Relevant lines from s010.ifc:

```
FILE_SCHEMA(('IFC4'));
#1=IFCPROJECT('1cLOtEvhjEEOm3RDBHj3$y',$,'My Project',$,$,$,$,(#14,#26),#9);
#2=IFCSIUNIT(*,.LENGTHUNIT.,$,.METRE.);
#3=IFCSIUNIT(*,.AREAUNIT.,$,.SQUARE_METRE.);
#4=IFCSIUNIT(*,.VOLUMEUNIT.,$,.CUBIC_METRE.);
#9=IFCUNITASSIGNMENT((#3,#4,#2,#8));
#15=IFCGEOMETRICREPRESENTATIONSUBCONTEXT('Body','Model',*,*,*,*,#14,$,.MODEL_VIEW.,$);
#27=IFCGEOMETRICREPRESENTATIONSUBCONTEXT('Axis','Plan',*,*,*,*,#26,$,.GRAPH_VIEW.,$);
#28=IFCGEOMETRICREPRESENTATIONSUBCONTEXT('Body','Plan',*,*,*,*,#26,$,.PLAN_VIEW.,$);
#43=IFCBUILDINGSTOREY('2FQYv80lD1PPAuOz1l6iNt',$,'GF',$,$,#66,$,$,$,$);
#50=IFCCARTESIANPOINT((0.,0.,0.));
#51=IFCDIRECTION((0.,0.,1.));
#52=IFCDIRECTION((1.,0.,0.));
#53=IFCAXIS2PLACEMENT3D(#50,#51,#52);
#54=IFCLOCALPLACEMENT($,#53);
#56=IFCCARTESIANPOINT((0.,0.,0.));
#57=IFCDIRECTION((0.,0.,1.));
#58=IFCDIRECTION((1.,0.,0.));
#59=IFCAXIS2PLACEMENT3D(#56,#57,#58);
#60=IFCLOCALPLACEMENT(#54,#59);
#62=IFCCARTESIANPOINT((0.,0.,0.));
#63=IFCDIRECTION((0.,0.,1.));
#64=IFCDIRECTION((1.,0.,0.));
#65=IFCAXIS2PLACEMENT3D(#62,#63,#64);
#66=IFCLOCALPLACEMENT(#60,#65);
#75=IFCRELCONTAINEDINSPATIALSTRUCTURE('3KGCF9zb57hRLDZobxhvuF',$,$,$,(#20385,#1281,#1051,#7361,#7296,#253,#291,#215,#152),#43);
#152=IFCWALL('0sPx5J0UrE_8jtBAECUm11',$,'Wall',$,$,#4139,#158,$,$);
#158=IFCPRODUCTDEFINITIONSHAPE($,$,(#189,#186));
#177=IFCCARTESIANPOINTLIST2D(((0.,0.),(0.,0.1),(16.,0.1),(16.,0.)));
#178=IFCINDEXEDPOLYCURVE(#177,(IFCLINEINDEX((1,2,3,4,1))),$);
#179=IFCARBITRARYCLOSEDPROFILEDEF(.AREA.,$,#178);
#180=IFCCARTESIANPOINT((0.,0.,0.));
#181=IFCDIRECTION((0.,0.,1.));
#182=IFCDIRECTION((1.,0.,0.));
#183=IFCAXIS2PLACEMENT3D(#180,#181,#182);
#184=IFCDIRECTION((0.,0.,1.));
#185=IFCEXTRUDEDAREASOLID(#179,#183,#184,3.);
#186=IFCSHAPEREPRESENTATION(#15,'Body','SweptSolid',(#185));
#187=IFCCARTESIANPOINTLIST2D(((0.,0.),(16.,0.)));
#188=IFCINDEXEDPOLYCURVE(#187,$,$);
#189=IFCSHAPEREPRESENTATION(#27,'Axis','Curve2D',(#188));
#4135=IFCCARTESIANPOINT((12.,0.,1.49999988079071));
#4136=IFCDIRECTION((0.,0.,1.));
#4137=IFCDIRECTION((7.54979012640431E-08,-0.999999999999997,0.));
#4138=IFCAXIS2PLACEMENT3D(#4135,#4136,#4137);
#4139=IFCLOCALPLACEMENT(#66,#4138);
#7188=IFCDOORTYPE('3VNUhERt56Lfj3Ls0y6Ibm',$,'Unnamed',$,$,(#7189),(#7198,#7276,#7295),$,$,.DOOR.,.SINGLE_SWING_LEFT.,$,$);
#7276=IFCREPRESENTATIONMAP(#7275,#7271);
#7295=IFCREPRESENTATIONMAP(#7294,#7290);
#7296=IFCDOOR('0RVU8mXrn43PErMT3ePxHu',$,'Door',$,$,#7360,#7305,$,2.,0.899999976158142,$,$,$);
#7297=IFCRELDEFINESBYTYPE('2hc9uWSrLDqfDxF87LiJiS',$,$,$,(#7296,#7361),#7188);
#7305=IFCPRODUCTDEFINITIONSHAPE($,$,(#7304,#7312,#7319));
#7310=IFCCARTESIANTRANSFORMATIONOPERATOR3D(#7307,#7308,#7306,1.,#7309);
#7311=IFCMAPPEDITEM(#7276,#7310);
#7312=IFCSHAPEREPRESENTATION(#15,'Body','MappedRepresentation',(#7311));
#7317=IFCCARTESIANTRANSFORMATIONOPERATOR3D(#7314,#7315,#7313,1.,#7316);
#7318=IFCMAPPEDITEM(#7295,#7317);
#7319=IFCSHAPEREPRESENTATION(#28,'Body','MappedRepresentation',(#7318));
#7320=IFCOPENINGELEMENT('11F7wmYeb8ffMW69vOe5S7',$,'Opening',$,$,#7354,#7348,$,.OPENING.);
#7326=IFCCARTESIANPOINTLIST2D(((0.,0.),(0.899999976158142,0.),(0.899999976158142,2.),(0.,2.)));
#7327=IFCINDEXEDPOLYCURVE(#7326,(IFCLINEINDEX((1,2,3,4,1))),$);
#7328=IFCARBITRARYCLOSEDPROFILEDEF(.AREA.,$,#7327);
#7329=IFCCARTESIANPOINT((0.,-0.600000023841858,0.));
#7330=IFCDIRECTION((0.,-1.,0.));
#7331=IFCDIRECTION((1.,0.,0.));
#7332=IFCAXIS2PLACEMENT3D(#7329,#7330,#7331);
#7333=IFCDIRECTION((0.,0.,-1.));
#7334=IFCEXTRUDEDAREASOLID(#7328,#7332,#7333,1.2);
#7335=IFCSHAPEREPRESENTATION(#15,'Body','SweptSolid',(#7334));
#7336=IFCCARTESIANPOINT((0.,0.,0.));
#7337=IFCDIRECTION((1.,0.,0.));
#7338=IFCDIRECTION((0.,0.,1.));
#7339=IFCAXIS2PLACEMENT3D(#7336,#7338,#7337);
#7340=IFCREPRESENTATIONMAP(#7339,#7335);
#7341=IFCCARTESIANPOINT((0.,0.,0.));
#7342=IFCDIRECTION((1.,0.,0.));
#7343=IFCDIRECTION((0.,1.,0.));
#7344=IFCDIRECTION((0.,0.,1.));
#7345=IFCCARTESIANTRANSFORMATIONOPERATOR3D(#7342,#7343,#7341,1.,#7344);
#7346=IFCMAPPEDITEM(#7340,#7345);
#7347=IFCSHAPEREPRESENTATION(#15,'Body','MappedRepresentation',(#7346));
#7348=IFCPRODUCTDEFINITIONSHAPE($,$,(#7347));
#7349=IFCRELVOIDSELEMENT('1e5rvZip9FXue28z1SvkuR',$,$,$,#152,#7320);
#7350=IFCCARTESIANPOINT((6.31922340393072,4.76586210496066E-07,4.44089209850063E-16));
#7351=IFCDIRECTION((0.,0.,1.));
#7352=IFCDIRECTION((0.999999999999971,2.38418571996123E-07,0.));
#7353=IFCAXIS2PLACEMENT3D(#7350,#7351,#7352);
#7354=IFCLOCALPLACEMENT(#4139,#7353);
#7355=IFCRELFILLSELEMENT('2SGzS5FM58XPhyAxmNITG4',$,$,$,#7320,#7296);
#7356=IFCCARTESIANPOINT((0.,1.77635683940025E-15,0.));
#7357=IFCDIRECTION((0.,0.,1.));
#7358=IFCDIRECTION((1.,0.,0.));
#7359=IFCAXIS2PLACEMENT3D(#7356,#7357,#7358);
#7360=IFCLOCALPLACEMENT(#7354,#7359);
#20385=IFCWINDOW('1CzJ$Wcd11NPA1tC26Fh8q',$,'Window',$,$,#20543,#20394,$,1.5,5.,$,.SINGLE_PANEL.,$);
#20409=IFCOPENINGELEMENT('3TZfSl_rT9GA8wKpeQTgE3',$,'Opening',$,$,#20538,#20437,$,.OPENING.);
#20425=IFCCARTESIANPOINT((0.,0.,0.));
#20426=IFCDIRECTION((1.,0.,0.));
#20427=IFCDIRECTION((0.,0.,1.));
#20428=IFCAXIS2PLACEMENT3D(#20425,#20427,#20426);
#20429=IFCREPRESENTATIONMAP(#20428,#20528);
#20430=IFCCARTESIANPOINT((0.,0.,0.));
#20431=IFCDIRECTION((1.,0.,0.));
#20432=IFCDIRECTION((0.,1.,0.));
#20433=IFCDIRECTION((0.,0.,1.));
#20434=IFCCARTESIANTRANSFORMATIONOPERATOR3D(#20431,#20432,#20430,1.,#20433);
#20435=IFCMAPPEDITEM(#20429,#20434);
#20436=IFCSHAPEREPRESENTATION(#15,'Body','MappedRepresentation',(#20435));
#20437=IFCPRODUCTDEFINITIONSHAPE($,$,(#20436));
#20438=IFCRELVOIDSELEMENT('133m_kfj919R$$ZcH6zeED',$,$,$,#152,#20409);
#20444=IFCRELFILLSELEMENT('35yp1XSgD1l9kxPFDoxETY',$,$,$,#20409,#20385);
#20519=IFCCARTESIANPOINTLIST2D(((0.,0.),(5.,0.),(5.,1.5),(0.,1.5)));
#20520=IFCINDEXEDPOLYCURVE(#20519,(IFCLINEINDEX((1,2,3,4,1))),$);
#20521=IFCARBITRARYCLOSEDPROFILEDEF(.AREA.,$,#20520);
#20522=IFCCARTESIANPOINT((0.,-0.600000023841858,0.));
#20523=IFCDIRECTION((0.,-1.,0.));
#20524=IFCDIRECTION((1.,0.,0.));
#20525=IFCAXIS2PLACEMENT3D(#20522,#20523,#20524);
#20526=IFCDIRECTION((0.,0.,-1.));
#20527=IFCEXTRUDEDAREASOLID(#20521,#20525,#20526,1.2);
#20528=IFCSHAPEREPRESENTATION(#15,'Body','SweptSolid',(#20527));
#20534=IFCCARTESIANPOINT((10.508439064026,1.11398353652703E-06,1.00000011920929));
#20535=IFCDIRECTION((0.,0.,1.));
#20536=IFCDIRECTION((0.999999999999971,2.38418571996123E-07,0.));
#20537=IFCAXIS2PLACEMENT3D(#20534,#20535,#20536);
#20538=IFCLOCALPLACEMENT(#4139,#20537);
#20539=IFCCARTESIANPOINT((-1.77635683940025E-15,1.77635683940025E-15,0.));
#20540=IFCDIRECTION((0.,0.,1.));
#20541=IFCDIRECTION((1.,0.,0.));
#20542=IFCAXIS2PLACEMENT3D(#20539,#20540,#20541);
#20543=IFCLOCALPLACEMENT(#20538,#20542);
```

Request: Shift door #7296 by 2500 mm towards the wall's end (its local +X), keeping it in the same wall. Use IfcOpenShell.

```python
import ifcopenshell
import ifcopenshell.api.geometry
import ifcopenshell.util.placement

model = ifcopenshell.open("s010.ifc")

door = model.by_guid("0RVU8mXrn43PErMT3ePxHu")
opening = door.FillsVoids[0].RelatingOpeningElement
wall = opening.VoidsElements[0].RelatingBuildingElement

wall_matrix = ifcopenshell.util.placement.get_local_placement(wall.ObjectPlacement)
shift = wall_matrix[:3, 0] * 2.5
before = ifcopenshell.util.placement.get_local_placement(door.ObjectPlacement)[:3, 3].copy()

# The door is placed relative to its opening, so it follows when the opening moves.
matrix = ifcopenshell.util.placement.get_local_placement(opening.ObjectPlacement)
matrix[:3, 3] += shift
ifcopenshell.api.geometry.edit_object_placement(
    model, product=opening, matrix=matrix, is_si=False, should_transform_children=True
)

after = ifcopenshell.util.placement.get_local_placement(door.ObjectPlacement)[:3, 3]
print("door moved by", (after - before).round(3) + 0.0)

model.write("s010_rev.ifc")
```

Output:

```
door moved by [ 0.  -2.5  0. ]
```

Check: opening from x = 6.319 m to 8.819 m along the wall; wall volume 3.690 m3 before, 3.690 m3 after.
